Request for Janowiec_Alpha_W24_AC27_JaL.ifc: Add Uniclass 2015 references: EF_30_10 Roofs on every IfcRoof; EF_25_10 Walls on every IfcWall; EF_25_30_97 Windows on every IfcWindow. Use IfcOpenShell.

First a look at what the model holds.

```python
import ifcopenshell

model = ifcopenshell.open("Janowiec_Alpha_W24_AC27_JaL.ifc")
print(model.schema)
print("classifications:", [c.Name for c in model.by_type("IfcClassification")])
for ifc_class in ("IfcDoor", "IfcRoof", "IfcStair", "IfcWall", "IfcWindow"):
    print(ifc_class, len(model.by_type(ifc_class)))
```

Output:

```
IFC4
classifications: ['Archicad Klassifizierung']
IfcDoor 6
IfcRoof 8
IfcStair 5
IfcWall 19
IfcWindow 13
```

```python
import ifcopenshell
import ifcopenshell.api.classification

model = ifcopenshell.open("Janowiec_Alpha_W24_AC27_JaL.ifc")

system = ifcopenshell.api.classification.add_classification(model, classification="Uniclass 2015")

codes = {
    "IfcRoof": ("EF_30_10", "Roofs"),
    "IfcWall": ("EF_25_10", "Walls"),
    "IfcWindow": ("EF_25_30_97", "Windows"),
}
for ifc_class, (code, name) in codes.items():
    products = model.by_type(ifc_class)
    ifcopenshell.api.classification.add_reference(
        model, products=products, classification=system, identification=code, name=name
    )
    print(code, len(products))

model.write("Janowiec_Alpha_W24_AC27_JaL_updated.ifc")
```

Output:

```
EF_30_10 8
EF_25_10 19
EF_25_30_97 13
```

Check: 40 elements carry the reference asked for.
